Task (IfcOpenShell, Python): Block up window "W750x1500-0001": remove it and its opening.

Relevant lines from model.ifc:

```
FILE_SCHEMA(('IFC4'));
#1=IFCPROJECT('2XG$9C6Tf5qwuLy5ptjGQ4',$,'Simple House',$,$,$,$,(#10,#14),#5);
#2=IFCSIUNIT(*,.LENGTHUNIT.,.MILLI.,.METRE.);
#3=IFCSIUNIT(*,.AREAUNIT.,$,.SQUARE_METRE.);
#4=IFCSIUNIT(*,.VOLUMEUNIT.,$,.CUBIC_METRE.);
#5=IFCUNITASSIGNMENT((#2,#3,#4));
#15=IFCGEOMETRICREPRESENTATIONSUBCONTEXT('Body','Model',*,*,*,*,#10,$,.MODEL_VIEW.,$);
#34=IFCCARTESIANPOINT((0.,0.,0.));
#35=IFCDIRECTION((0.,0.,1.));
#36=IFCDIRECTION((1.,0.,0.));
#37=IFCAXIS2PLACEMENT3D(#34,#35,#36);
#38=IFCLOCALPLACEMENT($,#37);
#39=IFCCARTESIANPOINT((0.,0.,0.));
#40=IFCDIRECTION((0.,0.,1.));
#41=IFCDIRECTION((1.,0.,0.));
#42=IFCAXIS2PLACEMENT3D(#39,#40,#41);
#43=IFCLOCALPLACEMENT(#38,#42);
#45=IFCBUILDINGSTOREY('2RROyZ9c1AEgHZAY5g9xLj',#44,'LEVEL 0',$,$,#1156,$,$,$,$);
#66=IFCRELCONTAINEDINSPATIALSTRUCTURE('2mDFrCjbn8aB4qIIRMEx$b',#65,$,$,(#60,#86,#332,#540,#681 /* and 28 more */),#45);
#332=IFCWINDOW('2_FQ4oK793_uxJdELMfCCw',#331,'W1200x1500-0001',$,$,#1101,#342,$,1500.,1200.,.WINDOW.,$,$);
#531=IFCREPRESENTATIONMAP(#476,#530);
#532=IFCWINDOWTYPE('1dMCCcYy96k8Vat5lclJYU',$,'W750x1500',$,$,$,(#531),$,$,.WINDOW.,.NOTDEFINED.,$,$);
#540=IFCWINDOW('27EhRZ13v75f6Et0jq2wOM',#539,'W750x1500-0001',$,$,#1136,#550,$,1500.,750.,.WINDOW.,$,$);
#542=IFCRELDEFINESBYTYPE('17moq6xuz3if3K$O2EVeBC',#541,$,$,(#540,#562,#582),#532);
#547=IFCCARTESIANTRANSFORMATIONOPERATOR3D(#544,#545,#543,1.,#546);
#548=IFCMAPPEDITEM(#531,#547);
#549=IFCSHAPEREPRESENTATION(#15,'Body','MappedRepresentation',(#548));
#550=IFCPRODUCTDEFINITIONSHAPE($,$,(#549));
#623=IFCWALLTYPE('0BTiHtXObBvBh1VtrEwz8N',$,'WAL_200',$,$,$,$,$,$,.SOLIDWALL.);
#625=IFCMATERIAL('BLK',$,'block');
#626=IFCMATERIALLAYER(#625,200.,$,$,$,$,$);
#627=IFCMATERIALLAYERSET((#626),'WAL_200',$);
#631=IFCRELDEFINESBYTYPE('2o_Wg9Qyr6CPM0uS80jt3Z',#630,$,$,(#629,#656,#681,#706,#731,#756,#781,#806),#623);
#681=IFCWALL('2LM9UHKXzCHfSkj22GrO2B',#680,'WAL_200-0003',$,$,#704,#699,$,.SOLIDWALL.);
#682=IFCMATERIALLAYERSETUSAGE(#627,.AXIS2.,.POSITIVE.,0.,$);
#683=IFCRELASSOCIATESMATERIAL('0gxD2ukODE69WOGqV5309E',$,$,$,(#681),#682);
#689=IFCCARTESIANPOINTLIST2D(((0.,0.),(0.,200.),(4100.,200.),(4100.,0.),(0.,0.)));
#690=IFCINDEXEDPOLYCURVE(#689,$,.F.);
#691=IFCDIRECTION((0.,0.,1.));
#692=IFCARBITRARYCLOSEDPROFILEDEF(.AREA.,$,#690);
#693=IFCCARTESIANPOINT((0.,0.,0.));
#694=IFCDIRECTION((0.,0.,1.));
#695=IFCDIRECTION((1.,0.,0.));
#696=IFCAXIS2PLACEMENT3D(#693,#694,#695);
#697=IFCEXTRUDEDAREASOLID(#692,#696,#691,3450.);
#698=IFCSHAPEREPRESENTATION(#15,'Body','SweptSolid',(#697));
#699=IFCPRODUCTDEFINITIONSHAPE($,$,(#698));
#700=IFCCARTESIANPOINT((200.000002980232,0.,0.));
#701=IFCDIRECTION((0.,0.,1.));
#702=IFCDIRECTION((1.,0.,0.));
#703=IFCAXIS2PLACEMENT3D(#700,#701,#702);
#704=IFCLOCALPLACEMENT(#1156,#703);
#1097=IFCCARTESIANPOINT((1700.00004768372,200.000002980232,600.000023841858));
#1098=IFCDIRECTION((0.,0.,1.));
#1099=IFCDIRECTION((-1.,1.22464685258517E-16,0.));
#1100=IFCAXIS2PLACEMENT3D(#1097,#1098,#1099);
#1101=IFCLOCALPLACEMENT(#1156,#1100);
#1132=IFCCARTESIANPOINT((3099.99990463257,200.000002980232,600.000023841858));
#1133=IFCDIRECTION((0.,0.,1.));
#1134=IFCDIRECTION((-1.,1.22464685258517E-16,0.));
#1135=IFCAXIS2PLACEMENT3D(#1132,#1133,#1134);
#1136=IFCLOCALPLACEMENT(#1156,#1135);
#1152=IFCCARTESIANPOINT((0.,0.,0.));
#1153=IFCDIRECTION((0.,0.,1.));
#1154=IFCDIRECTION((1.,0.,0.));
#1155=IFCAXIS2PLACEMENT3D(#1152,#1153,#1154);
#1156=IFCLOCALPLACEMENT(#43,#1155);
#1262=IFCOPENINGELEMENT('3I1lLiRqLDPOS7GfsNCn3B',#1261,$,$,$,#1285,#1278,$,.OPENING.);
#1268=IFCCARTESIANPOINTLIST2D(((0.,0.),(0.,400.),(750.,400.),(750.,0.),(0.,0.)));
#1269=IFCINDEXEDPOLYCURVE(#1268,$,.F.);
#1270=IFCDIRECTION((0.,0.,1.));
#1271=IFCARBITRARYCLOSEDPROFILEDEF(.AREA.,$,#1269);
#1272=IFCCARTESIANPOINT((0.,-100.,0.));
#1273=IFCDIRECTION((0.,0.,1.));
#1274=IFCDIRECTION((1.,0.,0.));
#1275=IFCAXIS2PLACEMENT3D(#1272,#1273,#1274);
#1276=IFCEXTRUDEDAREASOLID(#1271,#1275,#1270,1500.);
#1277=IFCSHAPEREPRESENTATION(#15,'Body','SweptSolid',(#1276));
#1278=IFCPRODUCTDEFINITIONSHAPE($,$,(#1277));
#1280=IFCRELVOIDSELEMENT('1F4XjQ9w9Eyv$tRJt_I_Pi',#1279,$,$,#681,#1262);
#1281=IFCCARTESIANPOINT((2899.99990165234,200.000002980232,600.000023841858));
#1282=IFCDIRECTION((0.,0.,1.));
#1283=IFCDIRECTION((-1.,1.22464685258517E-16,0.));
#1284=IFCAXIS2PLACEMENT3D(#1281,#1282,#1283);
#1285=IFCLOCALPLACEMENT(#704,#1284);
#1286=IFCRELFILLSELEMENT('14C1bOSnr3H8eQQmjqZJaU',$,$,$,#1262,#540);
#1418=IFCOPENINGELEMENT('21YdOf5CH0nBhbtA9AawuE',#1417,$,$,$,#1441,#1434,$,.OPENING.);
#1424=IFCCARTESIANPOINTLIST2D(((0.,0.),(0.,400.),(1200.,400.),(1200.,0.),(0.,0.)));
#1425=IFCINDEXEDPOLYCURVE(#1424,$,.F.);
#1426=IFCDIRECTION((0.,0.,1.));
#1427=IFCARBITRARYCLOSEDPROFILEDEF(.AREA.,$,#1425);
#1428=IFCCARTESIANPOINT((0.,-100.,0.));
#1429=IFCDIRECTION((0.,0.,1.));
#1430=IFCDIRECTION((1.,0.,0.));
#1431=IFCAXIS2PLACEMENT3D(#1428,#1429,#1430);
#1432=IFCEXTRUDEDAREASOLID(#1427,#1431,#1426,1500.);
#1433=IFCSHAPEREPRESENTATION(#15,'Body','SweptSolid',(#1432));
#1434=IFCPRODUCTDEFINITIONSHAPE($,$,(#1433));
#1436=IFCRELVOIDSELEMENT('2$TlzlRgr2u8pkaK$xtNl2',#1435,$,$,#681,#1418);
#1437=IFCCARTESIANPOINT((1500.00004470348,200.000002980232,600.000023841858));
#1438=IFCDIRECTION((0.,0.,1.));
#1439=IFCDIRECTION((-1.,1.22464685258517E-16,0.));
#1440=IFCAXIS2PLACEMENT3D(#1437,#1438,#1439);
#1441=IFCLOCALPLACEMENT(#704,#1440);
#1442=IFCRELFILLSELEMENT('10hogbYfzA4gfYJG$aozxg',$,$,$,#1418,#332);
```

```python
import ifcopenshell
import ifcopenshell.api.feature
import ifcopenshell.api.root
import ifcopenshell.geom
import ifcopenshell.util.shape

model = ifcopenshell.open("model.ifc")
settings = ifcopenshell.geom.settings()


def volume(element):
    """Net volume in cubic metres, openings subtracted."""
    shape = ifcopenshell.geom.create_shape(settings, element)
    return ifcopenshell.util.shape.get_volume(shape.geometry)


window = model.by_guid("27EhRZ13v75f6Et0jq2wOM")
opening = window.FillsVoids[0].RelatingOpeningElement
wall = opening.VoidsElements[0].RelatingBuildingElement
before = volume(wall)

ifcopenshell.api.root.remove_product(model, product=window)
ifcopenshell.api.feature.remove_feature(model, feature=opening)

after = volume(wall)

print(f"wall volume {before:.3f} -> {after:.3f} m3")

model.write("model_rev.ifc")
```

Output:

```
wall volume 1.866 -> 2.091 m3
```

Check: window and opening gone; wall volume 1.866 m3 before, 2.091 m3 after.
